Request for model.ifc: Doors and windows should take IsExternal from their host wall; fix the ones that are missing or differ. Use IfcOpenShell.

First a look at what the model holds.

```python
import ifcopenshell
import ifcopenshell.util.element

model = ifcopenshell.open("model.ifc")
print(model.schema)
seen = {}
for e in model.by_type("IfcDoor") + model.by_type("IfcWindow"):
    if not e.FillsVoids:
        continue
    host = e.FillsVoids[0].RelatingOpeningElement.VoidsElements[0].RelatingBuildingElement
    own = ifcopenshell.util.element.get_pset(e, f"Pset_{e.is_a()[3:].removesuffix('StandardCase')}Common", "IsExternal")
    wall = ifcopenshell.util.element.get_pset(host, "Pset_WallCommon", "IsExternal")
    seen[e.is_a(), own, wall] = seen.get((e.is_a(), own, wall), 0) + 1
for (cls, own, wall), count in sorted(seen.items(), key=str):
    print(count, cls, "IsExternal:", own, "| host wall:", wall)
```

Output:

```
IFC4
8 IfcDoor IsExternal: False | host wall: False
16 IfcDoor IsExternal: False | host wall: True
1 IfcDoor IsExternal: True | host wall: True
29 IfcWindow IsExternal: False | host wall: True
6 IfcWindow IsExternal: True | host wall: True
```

```python
import ifcopenshell
import ifcopenshell.api.pset
import ifcopenshell.util.element

model = ifcopenshell.open("model.ifc")

count = 0
for ifc_class, pset_name in (("IfcDoor", "Pset_DoorCommon"), ("IfcWindow", "Pset_WindowCommon")):
    for e in model.by_type(ifc_class):
        if not e.FillsVoids:
            continue
        host = e.FillsVoids[0].RelatingOpeningElement.VoidsElements[0].RelatingBuildingElement
        external = ifcopenshell.util.element.get_pset(host, "Pset_WallCommon", "IsExternal")
        if external is None or ifcopenshell.util.element.get_pset(e, pset_name, "IsExternal") == external:
            continue
        pset = ifcopenshell.api.pset.add_pset(model, product=e, name=pset_name)
        ifcopenshell.api.pset.edit_pset(model, pset=pset, properties={"IsExternal": external})
        count += 1

print(count, "updated")

model.write("model-out.ifc")
```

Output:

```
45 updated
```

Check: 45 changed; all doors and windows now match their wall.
